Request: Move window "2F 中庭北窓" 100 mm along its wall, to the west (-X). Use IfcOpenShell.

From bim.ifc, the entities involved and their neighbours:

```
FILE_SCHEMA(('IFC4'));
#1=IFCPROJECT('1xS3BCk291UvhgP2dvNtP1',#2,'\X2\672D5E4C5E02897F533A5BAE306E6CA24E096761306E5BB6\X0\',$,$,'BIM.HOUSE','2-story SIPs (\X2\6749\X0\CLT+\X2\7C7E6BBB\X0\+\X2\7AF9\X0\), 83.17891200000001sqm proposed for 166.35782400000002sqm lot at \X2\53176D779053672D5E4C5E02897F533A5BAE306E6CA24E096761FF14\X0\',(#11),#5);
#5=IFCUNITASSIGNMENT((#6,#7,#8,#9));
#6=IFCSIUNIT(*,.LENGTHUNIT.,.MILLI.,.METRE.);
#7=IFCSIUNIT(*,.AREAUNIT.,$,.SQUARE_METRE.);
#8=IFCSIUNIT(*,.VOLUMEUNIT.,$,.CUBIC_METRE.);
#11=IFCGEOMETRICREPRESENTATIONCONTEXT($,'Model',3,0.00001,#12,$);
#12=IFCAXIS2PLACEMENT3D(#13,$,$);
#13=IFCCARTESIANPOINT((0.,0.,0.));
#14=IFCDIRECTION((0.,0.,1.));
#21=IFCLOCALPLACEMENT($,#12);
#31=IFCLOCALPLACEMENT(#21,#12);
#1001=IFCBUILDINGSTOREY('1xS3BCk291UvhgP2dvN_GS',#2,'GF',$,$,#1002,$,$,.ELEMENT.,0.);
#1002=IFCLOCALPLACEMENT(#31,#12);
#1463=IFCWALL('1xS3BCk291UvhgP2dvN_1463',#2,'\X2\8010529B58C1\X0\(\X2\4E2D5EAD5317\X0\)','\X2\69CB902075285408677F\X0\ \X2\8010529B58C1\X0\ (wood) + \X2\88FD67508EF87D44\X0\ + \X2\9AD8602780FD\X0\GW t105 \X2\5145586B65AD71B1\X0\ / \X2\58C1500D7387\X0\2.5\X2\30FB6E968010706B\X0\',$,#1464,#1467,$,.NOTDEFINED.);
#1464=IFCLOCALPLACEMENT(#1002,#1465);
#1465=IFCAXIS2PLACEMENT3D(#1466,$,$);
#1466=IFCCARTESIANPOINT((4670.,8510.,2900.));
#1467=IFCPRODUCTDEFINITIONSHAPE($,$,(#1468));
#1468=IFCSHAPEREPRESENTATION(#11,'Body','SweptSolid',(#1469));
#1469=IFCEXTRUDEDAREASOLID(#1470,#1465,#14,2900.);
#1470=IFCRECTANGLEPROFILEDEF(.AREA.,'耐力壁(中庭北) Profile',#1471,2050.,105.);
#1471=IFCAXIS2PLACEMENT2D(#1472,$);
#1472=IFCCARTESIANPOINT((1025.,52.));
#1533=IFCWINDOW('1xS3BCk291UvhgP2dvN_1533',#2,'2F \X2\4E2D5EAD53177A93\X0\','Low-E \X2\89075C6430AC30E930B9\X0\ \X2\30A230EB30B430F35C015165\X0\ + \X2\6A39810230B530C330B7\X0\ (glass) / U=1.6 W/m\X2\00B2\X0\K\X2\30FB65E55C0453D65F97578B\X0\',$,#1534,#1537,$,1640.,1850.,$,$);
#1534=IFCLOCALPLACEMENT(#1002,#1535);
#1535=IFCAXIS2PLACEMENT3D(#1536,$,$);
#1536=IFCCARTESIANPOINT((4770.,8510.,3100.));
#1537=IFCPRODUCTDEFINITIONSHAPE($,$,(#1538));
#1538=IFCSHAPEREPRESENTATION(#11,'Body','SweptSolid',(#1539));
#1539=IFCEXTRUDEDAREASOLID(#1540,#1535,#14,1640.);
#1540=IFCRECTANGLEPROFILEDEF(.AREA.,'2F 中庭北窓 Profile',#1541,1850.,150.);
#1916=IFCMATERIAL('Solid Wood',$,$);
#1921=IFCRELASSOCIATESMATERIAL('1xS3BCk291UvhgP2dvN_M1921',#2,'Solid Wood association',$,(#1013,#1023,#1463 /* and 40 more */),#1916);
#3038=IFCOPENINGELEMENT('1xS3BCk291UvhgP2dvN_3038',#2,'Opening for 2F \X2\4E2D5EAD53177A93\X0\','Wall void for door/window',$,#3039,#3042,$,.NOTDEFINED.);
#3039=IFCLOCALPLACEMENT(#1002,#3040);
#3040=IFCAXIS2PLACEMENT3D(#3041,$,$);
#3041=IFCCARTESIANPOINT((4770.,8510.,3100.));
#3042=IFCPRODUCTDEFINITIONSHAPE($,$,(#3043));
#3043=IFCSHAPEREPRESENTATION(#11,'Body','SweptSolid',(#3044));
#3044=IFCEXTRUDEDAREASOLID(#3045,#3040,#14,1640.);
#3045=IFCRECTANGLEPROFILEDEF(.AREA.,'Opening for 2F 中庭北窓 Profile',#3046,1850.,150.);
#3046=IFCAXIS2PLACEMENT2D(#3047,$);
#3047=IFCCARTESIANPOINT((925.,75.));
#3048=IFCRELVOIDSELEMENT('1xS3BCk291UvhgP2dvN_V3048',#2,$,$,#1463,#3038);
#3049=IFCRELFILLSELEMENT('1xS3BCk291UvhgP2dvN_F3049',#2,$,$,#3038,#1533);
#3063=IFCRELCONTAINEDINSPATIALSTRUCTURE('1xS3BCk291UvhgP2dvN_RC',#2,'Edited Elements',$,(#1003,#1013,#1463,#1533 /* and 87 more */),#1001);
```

```python
import ifcopenshell
import ifcopenshell.api.geometry
import ifcopenshell.util.placement
import ifcopenshell.util.unit

model = ifcopenshell.open("bim.ifc")
unit_scale = ifcopenshell.util.unit.calculate_unit_scale(model)

window = model.by_id(1533)
opening = window.FillsVoids[0].RelatingOpeningElement
wall = opening.VoidsElements[0].RelatingBuildingElement

wall_matrix = ifcopenshell.util.placement.get_local_placement(wall.ObjectPlacement)
shift = wall_matrix[:3, 0] * -0.1 / unit_scale
before = ifcopenshell.util.placement.get_local_placement(window.ObjectPlacement)[:3, 3].copy()

# The window is not placed relative to its opening, so move both.
for product in (opening, window):
    matrix = ifcopenshell.util.placement.get_local_placement(product.ObjectPlacement)
    matrix[:3, 3] += shift
    ifcopenshell.api.geometry.edit_object_placement(model, product=product, matrix=matrix, is_si=False)

after = ifcopenshell.util.placement.get_local_placement(window.ObjectPlacement)[:3, 3]
print("window moved by", (after - before).round(3) + 0.0)

model.write("bim-out.ifc")
```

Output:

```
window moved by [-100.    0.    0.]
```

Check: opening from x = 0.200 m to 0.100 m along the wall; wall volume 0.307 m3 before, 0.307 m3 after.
